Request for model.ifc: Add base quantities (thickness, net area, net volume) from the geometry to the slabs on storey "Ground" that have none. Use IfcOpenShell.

First a look at what the model holds.

```python
import ifcopenshell
import ifcopenshell.util.element
import ifcopenshell.util.unit

model = ifcopenshell.open("model.ifc")
print(model.schema)
for unit_type in ("LENGTHUNIT", "AREAUNIT", "VOLUMEUNIT"):
    print(unit_type, ifcopenshell.util.unit.calculate_unit_scale(model, unit_type))
storey = next(s for s in model.by_type("IfcBuildingStorey") if s.Name == "Ground")
slabs = [e for e in ifcopenshell.util.element.get_decomposition(storey) if e.is_a("IfcSlab")]
for e in sorted(slabs, key=lambda e: e.id()):
    print(e.id(), e.is_a(), e.Name, list(ifcopenshell.util.element.get_psets(e, qtos_only=True)), sep=" | ")
```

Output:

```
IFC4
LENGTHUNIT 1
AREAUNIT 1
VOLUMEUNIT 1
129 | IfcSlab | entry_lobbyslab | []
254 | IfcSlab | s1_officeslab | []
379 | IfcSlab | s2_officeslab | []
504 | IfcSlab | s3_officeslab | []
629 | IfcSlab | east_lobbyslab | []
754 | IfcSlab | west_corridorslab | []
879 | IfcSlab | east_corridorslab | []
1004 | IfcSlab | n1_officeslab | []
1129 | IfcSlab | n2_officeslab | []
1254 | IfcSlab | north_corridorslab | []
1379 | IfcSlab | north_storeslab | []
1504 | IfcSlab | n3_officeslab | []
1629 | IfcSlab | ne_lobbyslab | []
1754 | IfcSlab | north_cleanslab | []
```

```python
import ifcopenshell
import ifcopenshell.api.pset
import ifcopenshell.geom
import ifcopenshell.util.element
import ifcopenshell.util.shape
import ifcopenshell.util.unit

model = ifcopenshell.open("model.ifc")
unit_scale = ifcopenshell.util.unit.calculate_unit_scale(model)
area_scale = ifcopenshell.util.unit.calculate_unit_scale(model, "AREAUNIT")
volume_scale = ifcopenshell.util.unit.calculate_unit_scale(model, "VOLUMEUNIT")
settings = ifcopenshell.geom.settings()

storey = next(s for s in model.by_type("IfcBuildingStorey") if s.Name == "Ground")
slabs = [e for e in ifcopenshell.util.element.get_decomposition(storey) if e.is_a("IfcSlab")]

for e in sorted(slabs, key=lambda e: e.id()):
    if ifcopenshell.util.element.get_psets(e, qtos_only=True, should_inherit=False):
        continue
    # Geometry comes back in metres, in the element's own axes.
    shape = ifcopenshell.geom.create_shape(settings, e)
    values = {
        "Width": ifcopenshell.util.shape.get_z(shape.geometry) / unit_scale,
        "NetArea": ifcopenshell.util.shape.get_footprint_area(shape.geometry) / area_scale,
        "NetVolume": ifcopenshell.util.shape.get_volume(shape.geometry) / volume_scale,
    }
    qto = ifcopenshell.api.pset.add_qto(model, product=e, name="Qto_SlabBaseQuantities")
    ifcopenshell.api.pset.edit_qto(model, qto=qto, properties=values)
    print(e.id(), {k: round(v, 3) for k, v in values.items()})

model.write("model_v2.ifc")
```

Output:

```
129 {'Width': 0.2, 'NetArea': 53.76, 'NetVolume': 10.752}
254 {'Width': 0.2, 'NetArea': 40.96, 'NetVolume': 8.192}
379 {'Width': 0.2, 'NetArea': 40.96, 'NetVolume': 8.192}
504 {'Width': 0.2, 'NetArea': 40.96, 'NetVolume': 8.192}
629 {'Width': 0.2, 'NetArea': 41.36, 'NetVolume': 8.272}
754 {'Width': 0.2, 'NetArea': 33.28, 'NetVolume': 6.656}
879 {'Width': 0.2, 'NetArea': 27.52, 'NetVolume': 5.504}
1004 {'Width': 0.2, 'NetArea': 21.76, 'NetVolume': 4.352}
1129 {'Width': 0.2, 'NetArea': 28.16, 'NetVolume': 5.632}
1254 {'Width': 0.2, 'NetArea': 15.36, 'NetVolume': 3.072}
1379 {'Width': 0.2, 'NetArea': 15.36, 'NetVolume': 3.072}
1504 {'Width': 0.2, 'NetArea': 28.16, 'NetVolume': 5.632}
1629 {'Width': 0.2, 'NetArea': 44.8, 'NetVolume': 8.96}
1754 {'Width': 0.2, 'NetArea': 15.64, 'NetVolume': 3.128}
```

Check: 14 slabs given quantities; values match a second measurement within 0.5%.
